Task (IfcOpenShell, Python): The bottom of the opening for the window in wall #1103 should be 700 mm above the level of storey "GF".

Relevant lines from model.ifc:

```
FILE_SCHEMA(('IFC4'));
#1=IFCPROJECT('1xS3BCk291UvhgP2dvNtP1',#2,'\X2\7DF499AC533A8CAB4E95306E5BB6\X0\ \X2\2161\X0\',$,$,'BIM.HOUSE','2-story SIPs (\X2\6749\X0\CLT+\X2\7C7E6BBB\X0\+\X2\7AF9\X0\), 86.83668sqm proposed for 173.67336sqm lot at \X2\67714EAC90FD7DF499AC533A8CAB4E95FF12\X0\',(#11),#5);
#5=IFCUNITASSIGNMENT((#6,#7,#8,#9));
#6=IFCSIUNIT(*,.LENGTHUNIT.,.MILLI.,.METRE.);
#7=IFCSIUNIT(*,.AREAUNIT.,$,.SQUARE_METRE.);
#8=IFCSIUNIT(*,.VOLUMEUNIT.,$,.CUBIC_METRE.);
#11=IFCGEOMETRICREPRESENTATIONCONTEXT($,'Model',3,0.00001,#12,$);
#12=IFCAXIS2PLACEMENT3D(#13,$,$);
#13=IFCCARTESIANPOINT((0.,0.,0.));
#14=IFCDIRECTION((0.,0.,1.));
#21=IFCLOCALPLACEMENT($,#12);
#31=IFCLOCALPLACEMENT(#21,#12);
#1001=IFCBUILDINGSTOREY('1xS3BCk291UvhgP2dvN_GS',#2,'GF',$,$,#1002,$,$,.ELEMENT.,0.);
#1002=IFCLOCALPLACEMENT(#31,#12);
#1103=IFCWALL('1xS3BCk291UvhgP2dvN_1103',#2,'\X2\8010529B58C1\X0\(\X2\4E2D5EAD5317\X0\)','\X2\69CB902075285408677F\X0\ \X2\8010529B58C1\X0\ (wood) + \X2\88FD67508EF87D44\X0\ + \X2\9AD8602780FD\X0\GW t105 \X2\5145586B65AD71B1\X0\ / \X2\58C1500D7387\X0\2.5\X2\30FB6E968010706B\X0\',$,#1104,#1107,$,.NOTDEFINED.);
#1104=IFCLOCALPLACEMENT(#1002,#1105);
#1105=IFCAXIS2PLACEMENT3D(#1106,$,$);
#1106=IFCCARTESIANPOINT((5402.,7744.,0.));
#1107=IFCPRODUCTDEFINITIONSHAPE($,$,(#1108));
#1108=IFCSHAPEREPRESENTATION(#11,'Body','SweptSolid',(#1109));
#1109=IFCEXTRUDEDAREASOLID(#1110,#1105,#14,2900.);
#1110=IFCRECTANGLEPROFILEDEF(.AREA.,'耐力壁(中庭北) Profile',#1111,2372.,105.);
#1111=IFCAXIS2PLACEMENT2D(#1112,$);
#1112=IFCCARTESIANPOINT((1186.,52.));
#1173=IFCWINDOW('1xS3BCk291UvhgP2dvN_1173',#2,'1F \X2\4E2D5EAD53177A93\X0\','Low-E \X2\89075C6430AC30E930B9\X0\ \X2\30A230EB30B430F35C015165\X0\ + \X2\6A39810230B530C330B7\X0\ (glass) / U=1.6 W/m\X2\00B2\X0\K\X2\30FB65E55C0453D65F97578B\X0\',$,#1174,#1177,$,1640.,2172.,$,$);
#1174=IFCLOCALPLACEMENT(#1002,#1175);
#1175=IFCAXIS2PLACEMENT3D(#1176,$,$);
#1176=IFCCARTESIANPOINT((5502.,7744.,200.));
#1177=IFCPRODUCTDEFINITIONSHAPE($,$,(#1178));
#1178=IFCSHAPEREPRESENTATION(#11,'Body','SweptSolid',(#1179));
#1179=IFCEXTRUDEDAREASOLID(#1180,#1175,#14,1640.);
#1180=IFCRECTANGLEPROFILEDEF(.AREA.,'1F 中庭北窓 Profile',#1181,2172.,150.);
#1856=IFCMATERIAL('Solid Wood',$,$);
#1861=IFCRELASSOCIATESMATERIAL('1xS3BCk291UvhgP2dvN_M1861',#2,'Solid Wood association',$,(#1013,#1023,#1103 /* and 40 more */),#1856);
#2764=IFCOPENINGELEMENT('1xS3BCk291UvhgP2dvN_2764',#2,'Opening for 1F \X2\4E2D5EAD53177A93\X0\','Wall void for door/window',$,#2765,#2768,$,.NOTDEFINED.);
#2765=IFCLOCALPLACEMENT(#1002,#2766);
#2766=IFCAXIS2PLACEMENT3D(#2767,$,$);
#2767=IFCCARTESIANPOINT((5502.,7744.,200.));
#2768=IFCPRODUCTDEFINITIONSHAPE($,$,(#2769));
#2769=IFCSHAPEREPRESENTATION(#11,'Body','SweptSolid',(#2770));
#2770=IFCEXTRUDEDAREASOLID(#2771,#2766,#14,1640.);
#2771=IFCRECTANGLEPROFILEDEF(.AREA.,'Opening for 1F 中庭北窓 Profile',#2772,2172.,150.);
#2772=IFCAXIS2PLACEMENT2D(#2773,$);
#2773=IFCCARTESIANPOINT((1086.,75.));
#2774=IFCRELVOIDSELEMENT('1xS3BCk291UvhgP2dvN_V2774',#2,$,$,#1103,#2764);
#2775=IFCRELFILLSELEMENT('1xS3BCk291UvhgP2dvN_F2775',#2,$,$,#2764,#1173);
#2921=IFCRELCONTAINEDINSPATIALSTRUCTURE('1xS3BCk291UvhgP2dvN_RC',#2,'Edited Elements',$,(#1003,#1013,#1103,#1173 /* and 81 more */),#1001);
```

```python
import numpy as np
import ifcopenshell
import ifcopenshell.api.geometry
import ifcopenshell.geom
import ifcopenshell.util.element
import ifcopenshell.util.placement
import ifcopenshell.util.shape
import ifcopenshell.util.unit

model = ifcopenshell.open("model.ifc")
unit_scale = ifcopenshell.util.unit.calculate_unit_scale(model)

window = model.by_guid("1xS3BCk291UvhgP2dvN_1173")
opening = window.FillsVoids[0].RelatingOpeningElement
storey = ifcopenshell.util.element.get_container(window, ifc_class="IfcBuildingStorey")
level = ifcopenshell.util.placement.get_local_placement(storey.ObjectPlacement)[2, 3]

# The opening's origin need not be at the sill, so measure its lowest point.
shape = ifcopenshell.geom.create_shape(ifcopenshell.geom.settings(), opening)
bottom = ifcopenshell.util.shape.get_shape_bottom_elevation(shape, shape.geometry) / unit_scale
dz = level + 0.7 / unit_scale - bottom

shift = np.array([0.0, 0.0, dz])
# The window is not placed relative to its opening, so move both.
for product in (opening, window):
    matrix = ifcopenshell.util.placement.get_local_placement(product.ObjectPlacement)
    matrix[:3, 3] += shift
    ifcopenshell.api.geometry.edit_object_placement(model, product=product, matrix=matrix, is_si=False)

print(f"moved by {dz * unit_scale:+.3f} m")

model.write("model_rev.ifc")
```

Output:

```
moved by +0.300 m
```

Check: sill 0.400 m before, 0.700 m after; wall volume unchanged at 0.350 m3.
